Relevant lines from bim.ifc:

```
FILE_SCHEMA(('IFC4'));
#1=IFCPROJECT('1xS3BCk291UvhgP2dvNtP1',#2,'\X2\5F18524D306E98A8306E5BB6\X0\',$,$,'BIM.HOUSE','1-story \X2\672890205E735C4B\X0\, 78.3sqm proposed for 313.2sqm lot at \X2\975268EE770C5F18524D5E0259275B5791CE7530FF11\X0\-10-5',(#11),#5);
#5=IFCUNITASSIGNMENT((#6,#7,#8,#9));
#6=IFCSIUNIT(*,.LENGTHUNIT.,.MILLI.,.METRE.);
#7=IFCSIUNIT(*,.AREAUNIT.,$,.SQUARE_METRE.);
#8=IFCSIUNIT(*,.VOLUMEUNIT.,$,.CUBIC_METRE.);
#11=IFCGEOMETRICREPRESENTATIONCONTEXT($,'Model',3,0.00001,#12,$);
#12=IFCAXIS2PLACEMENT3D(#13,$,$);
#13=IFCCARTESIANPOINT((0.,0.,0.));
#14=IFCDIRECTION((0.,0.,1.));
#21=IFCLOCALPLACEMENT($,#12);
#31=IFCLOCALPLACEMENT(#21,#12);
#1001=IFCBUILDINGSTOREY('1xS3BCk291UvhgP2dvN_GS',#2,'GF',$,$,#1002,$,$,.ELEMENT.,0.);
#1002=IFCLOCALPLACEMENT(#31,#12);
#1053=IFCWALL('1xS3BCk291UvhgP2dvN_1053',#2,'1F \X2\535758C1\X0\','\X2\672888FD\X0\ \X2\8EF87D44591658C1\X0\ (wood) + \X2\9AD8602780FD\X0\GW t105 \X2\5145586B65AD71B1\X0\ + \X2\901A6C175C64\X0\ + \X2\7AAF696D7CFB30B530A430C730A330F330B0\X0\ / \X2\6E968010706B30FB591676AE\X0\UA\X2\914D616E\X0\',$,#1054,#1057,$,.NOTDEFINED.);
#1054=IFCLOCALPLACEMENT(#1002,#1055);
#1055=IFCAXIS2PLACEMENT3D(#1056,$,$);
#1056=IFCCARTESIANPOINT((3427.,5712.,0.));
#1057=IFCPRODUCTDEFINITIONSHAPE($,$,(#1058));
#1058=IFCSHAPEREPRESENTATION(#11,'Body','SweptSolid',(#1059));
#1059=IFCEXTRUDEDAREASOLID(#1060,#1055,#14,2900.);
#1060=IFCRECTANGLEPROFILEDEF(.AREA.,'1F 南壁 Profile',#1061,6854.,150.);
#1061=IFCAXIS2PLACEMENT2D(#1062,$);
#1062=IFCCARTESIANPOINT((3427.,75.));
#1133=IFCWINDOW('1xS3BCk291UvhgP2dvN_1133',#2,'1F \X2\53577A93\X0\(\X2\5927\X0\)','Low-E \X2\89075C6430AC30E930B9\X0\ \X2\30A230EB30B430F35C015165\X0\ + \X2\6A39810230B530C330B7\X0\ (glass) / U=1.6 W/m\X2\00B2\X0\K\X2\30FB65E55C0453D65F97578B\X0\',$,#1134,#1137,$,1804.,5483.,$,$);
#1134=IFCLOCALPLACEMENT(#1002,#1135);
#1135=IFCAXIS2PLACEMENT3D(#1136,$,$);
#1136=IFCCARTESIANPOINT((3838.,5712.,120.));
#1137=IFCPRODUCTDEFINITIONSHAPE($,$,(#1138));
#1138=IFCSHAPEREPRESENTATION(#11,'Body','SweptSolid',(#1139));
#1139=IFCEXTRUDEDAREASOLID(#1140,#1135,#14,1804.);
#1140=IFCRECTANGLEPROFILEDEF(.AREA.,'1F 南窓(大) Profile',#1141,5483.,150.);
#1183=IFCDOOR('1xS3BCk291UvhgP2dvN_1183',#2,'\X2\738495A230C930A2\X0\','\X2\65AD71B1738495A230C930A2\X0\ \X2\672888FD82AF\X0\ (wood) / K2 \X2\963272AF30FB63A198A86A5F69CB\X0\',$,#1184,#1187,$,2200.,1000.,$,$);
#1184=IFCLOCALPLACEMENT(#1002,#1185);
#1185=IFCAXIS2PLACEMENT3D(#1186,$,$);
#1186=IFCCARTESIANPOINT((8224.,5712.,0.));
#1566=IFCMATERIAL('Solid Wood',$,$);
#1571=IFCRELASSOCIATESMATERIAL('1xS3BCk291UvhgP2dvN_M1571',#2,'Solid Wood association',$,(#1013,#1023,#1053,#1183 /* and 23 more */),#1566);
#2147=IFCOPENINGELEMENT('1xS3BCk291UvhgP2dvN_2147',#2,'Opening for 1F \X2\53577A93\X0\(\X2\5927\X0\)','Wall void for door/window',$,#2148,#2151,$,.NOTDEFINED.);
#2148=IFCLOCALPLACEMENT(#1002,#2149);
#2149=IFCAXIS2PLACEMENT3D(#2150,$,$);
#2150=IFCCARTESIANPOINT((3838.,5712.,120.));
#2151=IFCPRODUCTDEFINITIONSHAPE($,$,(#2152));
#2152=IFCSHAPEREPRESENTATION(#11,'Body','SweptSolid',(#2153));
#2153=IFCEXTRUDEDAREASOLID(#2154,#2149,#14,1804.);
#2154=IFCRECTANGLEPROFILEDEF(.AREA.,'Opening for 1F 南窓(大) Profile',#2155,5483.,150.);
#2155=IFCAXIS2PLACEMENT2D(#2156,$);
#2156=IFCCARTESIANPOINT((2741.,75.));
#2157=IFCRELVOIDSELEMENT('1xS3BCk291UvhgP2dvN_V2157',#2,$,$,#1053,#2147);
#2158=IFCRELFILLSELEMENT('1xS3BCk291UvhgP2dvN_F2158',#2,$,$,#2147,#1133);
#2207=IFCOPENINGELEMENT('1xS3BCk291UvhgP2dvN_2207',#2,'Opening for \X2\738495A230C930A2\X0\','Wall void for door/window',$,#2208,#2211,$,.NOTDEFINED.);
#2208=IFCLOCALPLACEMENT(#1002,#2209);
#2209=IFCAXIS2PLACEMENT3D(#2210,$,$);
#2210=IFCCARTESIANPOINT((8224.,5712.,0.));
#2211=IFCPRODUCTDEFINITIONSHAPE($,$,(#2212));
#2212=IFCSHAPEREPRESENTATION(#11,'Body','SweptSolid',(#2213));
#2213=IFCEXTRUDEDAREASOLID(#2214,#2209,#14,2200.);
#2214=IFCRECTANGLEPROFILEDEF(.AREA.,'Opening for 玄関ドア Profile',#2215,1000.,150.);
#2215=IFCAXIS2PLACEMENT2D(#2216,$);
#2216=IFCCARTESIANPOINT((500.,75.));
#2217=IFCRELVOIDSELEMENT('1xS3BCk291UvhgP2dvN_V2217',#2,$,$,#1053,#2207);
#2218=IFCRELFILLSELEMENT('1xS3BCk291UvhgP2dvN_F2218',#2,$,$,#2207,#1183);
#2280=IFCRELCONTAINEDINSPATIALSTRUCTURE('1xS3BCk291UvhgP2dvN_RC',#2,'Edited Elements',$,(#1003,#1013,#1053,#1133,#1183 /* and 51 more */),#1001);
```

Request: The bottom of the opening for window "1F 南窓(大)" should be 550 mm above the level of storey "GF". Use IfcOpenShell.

```python
import numpy as np
import ifcopenshell
import ifcopenshell.api.geometry
import ifcopenshell.geom
import ifcopenshell.util.element
import ifcopenshell.util.placement
import ifcopenshell.util.shape
import ifcopenshell.util.unit

model = ifcopenshell.open("bim.ifc")
unit_scale = ifcopenshell.util.unit.calculate_unit_scale(model)

window = model.by_id(1133)
opening = window.FillsVoids[0].RelatingOpeningElement
storey = ifcopenshell.util.element.get_container(window, ifc_class="IfcBuildingStorey")
level = ifcopenshell.util.placement.get_local_placement(storey.ObjectPlacement)[2, 3]

# The opening's origin need not be at the sill, so measure its lowest point.
shape = ifcopenshell.geom.create_shape(ifcopenshell.geom.settings(), opening)
bottom = ifcopenshell.util.shape.get_shape_bottom_elevation(shape, shape.geometry) / unit_scale
dz = level + 550.0 - bottom

shift = np.array([0.0, 0.0, dz])
# The window is not placed relative to its opening, so move both.
for product in (opening, window):
    matrix = ifcopenshell.util.placement.get_local_placement(product.ObjectPlacement)
    matrix[:3, 3] += shift
    ifcopenshell.api.geometry.edit_object_placement(model, product=product, matrix=matrix, is_si=False)

print(f"moved by {dz * unit_scale:+.3f} m")

model.write("bim_edited.ifc")
```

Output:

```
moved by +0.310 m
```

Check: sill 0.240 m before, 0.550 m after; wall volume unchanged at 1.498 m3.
